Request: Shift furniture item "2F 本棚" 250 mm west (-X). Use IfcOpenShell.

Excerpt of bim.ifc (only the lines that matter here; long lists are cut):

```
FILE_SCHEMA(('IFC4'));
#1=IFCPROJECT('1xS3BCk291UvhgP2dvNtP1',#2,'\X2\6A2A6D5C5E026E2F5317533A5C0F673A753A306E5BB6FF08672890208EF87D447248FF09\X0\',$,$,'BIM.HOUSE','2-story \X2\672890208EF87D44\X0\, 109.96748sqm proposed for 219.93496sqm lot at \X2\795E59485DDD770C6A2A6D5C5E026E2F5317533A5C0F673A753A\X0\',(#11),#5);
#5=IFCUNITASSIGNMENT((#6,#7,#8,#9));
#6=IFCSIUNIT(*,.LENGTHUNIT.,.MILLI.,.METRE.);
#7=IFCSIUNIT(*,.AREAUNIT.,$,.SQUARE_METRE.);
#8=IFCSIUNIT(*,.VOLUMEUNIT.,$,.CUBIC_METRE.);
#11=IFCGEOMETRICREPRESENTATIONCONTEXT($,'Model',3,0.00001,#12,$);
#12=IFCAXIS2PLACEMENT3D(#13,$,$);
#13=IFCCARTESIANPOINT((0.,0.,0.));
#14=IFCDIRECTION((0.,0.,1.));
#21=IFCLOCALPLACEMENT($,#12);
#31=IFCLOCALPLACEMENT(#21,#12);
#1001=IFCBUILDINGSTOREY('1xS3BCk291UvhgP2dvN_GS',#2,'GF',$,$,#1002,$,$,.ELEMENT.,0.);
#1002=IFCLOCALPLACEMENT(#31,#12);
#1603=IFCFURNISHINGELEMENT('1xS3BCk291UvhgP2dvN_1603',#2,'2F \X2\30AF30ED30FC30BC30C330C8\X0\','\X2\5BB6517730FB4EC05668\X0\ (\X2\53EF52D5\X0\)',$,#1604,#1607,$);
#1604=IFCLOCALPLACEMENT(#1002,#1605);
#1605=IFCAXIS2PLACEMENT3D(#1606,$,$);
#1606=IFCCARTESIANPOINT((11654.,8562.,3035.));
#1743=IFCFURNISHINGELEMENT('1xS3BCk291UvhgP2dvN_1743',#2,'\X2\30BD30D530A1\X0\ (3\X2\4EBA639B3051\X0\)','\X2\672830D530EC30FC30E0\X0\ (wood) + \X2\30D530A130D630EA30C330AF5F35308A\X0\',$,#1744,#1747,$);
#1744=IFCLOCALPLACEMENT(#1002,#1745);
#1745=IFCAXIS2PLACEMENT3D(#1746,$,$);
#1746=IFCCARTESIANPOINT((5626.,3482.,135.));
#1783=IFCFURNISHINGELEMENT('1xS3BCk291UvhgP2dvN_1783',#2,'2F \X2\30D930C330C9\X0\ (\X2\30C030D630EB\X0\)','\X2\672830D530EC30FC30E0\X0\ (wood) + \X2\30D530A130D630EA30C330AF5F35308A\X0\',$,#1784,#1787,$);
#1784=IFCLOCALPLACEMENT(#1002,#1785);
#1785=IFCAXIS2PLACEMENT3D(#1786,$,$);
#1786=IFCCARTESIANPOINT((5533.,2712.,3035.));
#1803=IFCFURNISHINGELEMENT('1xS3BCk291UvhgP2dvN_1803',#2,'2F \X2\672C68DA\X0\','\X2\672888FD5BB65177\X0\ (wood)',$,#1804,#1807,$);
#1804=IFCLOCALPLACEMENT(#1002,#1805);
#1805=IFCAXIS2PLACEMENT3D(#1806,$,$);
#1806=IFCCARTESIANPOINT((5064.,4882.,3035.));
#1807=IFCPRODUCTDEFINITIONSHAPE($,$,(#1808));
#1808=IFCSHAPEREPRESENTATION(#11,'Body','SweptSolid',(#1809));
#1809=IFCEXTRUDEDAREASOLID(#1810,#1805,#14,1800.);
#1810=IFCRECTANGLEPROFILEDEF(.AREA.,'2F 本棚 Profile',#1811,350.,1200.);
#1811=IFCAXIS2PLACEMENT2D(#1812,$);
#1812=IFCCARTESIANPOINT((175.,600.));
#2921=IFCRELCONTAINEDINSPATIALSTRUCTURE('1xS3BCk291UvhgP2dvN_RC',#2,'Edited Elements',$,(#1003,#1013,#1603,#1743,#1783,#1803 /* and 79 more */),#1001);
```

```python
import ifcopenshell
import ifcopenshell.api.geometry
import ifcopenshell.util.placement

model = ifcopenshell.open("bim.ifc")

item = model.by_guid("1xS3BCk291UvhgP2dvN_1803")
matrix = ifcopenshell.util.placement.get_local_placement(item.ObjectPlacement)
matrix[0, 3] -= 250.0
ifcopenshell.api.geometry.edit_object_placement(model, product=item, matrix=matrix, is_si=False)

print(ifcopenshell.util.placement.get_local_placement(item.ObjectPlacement).round(3) + 0.0)

model.write("bim_updated.ifc")
```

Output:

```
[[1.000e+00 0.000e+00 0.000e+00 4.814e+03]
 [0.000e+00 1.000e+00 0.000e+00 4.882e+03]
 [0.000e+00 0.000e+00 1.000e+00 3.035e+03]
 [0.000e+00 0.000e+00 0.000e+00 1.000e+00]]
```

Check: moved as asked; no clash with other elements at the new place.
